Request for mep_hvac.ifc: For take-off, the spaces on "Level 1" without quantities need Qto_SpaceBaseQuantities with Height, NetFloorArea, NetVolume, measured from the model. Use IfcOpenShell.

First a look at what the model holds.

```python
import ifcopenshell
import ifcopenshell.util.element
import ifcopenshell.util.unit

model = ifcopenshell.open("mep_hvac.ifc")
print(model.schema)
for unit_type in ("LENGTHUNIT", "AREAUNIT", "VOLUMEUNIT"):
    print(unit_type, ifcopenshell.util.unit.calculate_unit_scale(model, unit_type))
storey = next(s for s in model.by_type("IfcBuildingStorey") if s.Name == "Level 1")
spaces = [e for e in ifcopenshell.util.element.get_decomposition(storey) if e.is_a("IfcSpace")]
for e in sorted(spaces, key=lambda e: e.id()):
    print(e.id(), e.is_a(), e.Name, list(ifcopenshell.util.element.get_psets(e, qtos_only=True)), sep=" | ")
```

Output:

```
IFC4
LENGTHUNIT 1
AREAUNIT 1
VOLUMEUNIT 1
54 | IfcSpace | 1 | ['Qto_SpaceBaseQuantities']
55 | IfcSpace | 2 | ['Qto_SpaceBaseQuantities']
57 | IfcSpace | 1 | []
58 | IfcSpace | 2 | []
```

```python
import ifcopenshell
import ifcopenshell.api.pset
import ifcopenshell.geom
import ifcopenshell.util.element
import ifcopenshell.util.shape
import ifcopenshell.util.unit

model = ifcopenshell.open("mep_hvac.ifc")
unit_scale = ifcopenshell.util.unit.calculate_unit_scale(model)
area_scale = ifcopenshell.util.unit.calculate_unit_scale(model, "AREAUNIT")
volume_scale = ifcopenshell.util.unit.calculate_unit_scale(model, "VOLUMEUNIT")
settings = ifcopenshell.geom.settings()

storey = next(s for s in model.by_type("IfcBuildingStorey") if s.Name == "Level 1")
spaces = [e for e in ifcopenshell.util.element.get_decomposition(storey) if e.is_a("IfcSpace")]

for e in sorted(spaces, key=lambda e: e.id()):
    if ifcopenshell.util.element.get_psets(e, qtos_only=True, should_inherit=False):
        continue
    # Geometry comes back in metres, in the element's own axes.
    shape = ifcopenshell.geom.create_shape(settings, e)
    values = {
        "Height": ifcopenshell.util.shape.get_z(shape.geometry) / unit_scale,
        "NetFloorArea": ifcopenshell.util.shape.get_footprint_area(shape.geometry) / area_scale,
        "NetVolume": ifcopenshell.util.shape.get_volume(shape.geometry) / volume_scale,
    }
    qto = ifcopenshell.api.pset.add_qto(model, product=e, name="Qto_SpaceBaseQuantities")
    ifcopenshell.api.pset.edit_qto(model, qto=qto, properties=values)
    print(e.id(), {k: round(v, 3) for k, v in values.items()})

model.write("mep_hvac_edited.ifc")
```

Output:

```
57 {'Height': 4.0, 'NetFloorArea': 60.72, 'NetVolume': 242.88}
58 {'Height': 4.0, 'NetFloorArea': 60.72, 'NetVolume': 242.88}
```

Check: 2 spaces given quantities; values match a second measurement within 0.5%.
